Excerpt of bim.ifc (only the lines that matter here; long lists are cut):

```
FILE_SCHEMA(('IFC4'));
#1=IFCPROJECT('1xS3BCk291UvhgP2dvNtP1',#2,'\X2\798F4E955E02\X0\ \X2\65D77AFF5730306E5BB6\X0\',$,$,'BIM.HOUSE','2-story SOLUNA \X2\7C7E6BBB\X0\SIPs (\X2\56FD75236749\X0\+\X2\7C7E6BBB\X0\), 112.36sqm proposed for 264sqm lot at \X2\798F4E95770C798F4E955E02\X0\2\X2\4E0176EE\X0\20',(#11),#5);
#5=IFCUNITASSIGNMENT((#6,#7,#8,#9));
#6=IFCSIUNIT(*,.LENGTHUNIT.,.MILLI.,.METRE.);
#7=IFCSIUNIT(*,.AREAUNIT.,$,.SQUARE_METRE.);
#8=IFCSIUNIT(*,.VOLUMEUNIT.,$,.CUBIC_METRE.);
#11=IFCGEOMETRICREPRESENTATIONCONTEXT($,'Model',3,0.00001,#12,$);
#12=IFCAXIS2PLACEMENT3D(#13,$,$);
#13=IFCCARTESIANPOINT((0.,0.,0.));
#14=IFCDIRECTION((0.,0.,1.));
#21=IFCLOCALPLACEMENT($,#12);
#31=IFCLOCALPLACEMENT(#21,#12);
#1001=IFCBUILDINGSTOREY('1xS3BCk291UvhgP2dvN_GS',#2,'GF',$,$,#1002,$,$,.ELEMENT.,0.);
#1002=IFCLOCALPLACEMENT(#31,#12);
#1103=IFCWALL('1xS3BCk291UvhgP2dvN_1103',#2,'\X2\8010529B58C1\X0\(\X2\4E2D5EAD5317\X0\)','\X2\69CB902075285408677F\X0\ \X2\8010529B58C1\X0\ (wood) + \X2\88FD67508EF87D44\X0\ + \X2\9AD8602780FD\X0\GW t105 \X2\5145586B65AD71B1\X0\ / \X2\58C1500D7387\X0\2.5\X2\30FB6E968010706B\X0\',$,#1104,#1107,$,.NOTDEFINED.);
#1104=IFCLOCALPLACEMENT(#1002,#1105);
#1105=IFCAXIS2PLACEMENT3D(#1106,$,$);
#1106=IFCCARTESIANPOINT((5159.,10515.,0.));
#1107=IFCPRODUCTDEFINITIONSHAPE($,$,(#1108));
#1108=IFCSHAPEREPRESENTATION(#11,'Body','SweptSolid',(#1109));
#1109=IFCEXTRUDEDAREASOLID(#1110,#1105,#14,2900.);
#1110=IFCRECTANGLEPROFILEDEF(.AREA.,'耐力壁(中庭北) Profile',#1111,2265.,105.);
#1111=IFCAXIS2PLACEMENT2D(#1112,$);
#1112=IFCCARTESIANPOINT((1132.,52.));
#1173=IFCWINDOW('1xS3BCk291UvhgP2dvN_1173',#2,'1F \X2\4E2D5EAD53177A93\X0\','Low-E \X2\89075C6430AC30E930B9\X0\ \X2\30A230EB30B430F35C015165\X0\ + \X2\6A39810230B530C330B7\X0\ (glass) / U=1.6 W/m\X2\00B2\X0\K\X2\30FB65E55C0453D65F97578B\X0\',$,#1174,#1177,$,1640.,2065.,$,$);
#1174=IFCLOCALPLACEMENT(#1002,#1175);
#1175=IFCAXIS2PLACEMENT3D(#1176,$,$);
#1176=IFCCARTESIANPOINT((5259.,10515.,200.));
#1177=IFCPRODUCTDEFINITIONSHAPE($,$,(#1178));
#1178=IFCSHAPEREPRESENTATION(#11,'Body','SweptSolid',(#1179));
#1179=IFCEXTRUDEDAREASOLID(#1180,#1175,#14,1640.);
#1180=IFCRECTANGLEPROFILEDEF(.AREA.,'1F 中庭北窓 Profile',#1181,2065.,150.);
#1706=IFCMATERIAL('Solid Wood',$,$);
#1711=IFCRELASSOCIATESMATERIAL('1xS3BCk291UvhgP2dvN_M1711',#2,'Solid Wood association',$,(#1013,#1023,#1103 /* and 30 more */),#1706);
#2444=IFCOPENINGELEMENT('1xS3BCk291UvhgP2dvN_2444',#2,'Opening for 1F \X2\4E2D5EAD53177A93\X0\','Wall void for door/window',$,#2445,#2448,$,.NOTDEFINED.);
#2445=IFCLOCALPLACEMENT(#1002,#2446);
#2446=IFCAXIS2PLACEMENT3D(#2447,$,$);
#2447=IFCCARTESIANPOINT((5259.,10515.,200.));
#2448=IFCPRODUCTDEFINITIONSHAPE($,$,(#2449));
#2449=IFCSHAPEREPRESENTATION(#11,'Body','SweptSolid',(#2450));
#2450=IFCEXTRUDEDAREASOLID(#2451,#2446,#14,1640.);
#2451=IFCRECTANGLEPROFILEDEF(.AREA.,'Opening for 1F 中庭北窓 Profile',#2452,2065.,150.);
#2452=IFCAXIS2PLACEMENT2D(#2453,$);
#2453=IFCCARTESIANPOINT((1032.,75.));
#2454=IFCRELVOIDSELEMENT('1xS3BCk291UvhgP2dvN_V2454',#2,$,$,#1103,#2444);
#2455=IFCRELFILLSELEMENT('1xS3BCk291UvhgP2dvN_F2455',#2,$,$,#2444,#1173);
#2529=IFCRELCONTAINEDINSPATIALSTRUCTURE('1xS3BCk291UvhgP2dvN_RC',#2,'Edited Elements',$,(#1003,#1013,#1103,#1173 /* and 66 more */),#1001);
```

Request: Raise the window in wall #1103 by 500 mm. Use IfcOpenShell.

```python
import numpy as np
import ifcopenshell
import ifcopenshell.api.geometry
import ifcopenshell.util.placement
import ifcopenshell.util.unit

model = ifcopenshell.open("bim.ifc")
unit_scale = ifcopenshell.util.unit.calculate_unit_scale(model)

window = model.by_guid("1xS3BCk291UvhgP2dvN_1173")
opening = window.FillsVoids[0].RelatingOpeningElement
dz = 500.0

shift = np.array([0.0, 0.0, dz])
# The window is not placed relative to its opening, so move both.
for product in (opening, window):
    matrix = ifcopenshell.util.placement.get_local_placement(product.ObjectPlacement)
    matrix[:3, 3] += shift
    ifcopenshell.api.geometry.edit_object_placement(model, product=product, matrix=matrix, is_si=False)

print(f"moved by {dz * unit_scale:+.3f} m")

model.write("bim_v2.ifc")
```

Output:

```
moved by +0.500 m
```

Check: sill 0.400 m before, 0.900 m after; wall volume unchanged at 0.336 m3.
